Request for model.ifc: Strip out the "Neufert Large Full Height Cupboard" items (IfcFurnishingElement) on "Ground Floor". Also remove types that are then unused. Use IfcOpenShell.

First a look at what the model holds.

```python
import ifcopenshell
import ifcopenshell.util.element

model = ifcopenshell.open("model.ifc")
print(model.schema)
storey = next(s for s in model.by_type("IfcBuildingStorey") if s.Name == "Ground Floor")
furniture = [e for e in ifcopenshell.util.element.get_decomposition(storey) if e.is_a("IfcFurnishingElement")]
seen = {}
for e in furniture:
    element_type = ifcopenshell.util.element.get_type(e)
    name = element_type.Name if element_type not in (None, e) else None
    seen[name] = seen.get(name, 0) + 1
for name, count in sorted(seen.items(), key=str):
    print(count, "x", name)
```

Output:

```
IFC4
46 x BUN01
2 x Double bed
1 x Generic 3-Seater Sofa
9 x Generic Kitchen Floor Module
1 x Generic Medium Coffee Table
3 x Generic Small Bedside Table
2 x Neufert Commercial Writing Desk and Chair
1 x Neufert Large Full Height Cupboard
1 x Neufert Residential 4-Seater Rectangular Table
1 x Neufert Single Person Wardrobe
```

```python
import ifcopenshell
import ifcopenshell.api.root
import ifcopenshell.util.element

model = ifcopenshell.open("model.ifc")

storey = next(s for s in model.by_type("IfcBuildingStorey") if s.Name == "Ground Floor")
furniture = [e for e in ifcopenshell.util.element.get_decomposition(storey) if e.is_a("IfcFurnishingElement")]
targets = [e for e in furniture if (t := ifcopenshell.util.element.get_type(e)) not in (None, e) and t.Name == "Neufert Large Full Height Cupboard"]
types = {ifcopenshell.util.element.get_type(e) for e in targets} - {None, *targets}

for e in targets:
    ifcopenshell.api.root.remove_product(model, product=e)
print(len(targets), "removed")

unused = [t for t in types if not ifcopenshell.util.element.get_types(t)]
for t in unused:
    ifcopenshell.api.root.remove_product(model, product=t)
print(len(unused), "unused types removed")

model.write("model_rev.ifc")
```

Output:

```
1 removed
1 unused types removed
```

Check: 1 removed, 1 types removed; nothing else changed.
